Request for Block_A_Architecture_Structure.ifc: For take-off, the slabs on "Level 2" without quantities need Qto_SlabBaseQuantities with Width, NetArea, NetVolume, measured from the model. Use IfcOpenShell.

First a look at what the model holds.

```python
import ifcopenshell
import ifcopenshell.util.element
import ifcopenshell.util.unit

model = ifcopenshell.open("Block_A_Architecture_Structure.ifc")
print(model.schema)
for unit_type in ("LENGTHUNIT", "AREAUNIT", "VOLUMEUNIT"):
    print(unit_type, ifcopenshell.util.unit.calculate_unit_scale(model, unit_type))
storey = next(s for s in model.by_type("IfcBuildingStorey") if s.Name == "Level 2")
slabs = [e for e in ifcopenshell.util.element.get_decomposition(storey) if e.is_a("IfcSlab")]
for e in sorted(slabs, key=lambda e: e.id()):
    print(e.id(), e.is_a(), e.Name, list(ifcopenshell.util.element.get_psets(e, qtos_only=True)), sep=" | ")
```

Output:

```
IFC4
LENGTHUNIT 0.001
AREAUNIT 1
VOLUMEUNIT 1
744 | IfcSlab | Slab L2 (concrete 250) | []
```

```python
import ifcopenshell
import ifcopenshell.api.pset
import ifcopenshell.geom
import ifcopenshell.util.element
import ifcopenshell.util.shape
import ifcopenshell.util.unit

model = ifcopenshell.open("Block_A_Architecture_Structure.ifc")
unit_scale = ifcopenshell.util.unit.calculate_unit_scale(model)
area_scale = ifcopenshell.util.unit.calculate_unit_scale(model, "AREAUNIT")
volume_scale = ifcopenshell.util.unit.calculate_unit_scale(model, "VOLUMEUNIT")
settings = ifcopenshell.geom.settings()

storey = next(s for s in model.by_type("IfcBuildingStorey") if s.Name == "Level 2")
slabs = [e for e in ifcopenshell.util.element.get_decomposition(storey) if e.is_a("IfcSlab")]

for e in sorted(slabs, key=lambda e: e.id()):
    if ifcopenshell.util.element.get_psets(e, qtos_only=True, should_inherit=False):
        continue
    # Geometry comes back in metres, in the element's own axes.
    shape = ifcopenshell.geom.create_shape(settings, e)
    values = {
        "Width": ifcopenshell.util.shape.get_z(shape.geometry) / unit_scale,
        "NetArea": ifcopenshell.util.shape.get_footprint_area(shape.geometry) / area_scale,
        "NetVolume": ifcopenshell.util.shape.get_volume(shape.geometry) / volume_scale,
    }
    qto = ifcopenshell.api.pset.add_qto(model, product=e, name="Qto_SlabBaseQuantities")
    ifcopenshell.api.pset.edit_qto(model, qto=qto, properties=values)
    print(e.id(), {k: round(v, 3) for k, v in values.items()})

model.write("Block_A_Architecture_Structure_updated.ifc")
```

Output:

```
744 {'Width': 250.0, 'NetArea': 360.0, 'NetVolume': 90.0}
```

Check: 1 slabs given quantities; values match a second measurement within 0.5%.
